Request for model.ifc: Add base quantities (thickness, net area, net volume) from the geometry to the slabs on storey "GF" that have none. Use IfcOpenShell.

First a look at what the model holds.

```python
import ifcopenshell
import ifcopenshell.util.element
import ifcopenshell.util.unit

model = ifcopenshell.open("model.ifc")
print(model.schema)
for unit_type in ("LENGTHUNIT", "AREAUNIT", "VOLUMEUNIT"):
    print(unit_type, ifcopenshell.util.unit.calculate_unit_scale(model, unit_type))
storey = next(s for s in model.by_type("IfcBuildingStorey") if s.Name == "GF")
slabs = [e for e in ifcopenshell.util.element.get_decomposition(storey) if e.is_a("IfcSlab")]
for e in sorted(slabs, key=lambda e: e.id()):
    print(e.id(), e.is_a(), e.Name, list(ifcopenshell.util.element.get_psets(e, qtos_only=True)), sep=" | ")
```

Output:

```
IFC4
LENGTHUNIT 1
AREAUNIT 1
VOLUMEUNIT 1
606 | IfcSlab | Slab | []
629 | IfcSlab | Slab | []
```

```python
import ifcopenshell
import ifcopenshell.api.pset
import ifcopenshell.geom
import ifcopenshell.util.element
import ifcopenshell.util.shape
import ifcopenshell.util.unit

model = ifcopenshell.open("model.ifc")
unit_scale = ifcopenshell.util.unit.calculate_unit_scale(model)
area_scale = ifcopenshell.util.unit.calculate_unit_scale(model, "AREAUNIT")
volume_scale = ifcopenshell.util.unit.calculate_unit_scale(model, "VOLUMEUNIT")
settings = ifcopenshell.geom.settings()

storey = next(s for s in model.by_type("IfcBuildingStorey") if s.Name == "GF")
slabs = [e for e in ifcopenshell.util.element.get_decomposition(storey) if e.is_a("IfcSlab")]

for e in sorted(slabs, key=lambda e: e.id()):
    if ifcopenshell.util.element.get_psets(e, qtos_only=True, should_inherit=False):
        continue
    # Geometry comes back in metres, in the element's own axes.
    shape = ifcopenshell.geom.create_shape(settings, e)
    values = {
        "Width": ifcopenshell.util.shape.get_z(shape.geometry) / unit_scale,
        "NetArea": ifcopenshell.util.shape.get_footprint_area(shape.geometry) / area_scale,
        "NetVolume": ifcopenshell.util.shape.get_volume(shape.geometry) / volume_scale,
    }
    qto = ifcopenshell.api.pset.add_qto(model, product=e, name="Qto_SlabBaseQuantities")
    ifcopenshell.api.pset.edit_qto(model, qto=qto, properties=values)
    print(e.id(), {k: round(v, 3) for k, v in values.items()})

model.write("model_v2.ifc")
```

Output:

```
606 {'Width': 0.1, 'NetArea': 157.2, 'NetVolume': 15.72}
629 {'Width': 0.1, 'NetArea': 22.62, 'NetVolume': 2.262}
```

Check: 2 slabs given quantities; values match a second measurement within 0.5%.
